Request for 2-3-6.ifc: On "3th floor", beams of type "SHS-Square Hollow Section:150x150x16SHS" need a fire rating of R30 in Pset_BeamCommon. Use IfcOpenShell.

First a look at what the model holds.

```python
import ifcopenshell
import ifcopenshell.util.element

model = ifcopenshell.open("2-3-6.ifc")
print(model.schema)
storey = next(s for s in model.by_type("IfcBuildingStorey") if s.Name == "3th floor")
beams = [e for e in ifcopenshell.util.element.get_decomposition(storey) if e.is_a("IfcBeam")]
seen = {}
for e in beams:
    element_type = ifcopenshell.util.element.get_type(e)
    key = (element_type.Name if element_type != e and element_type else None, ifcopenshell.util.element.get_pset(e, "Pset_BeamCommon", "FireRating"))
    seen[key] = seen.get(key, 0) + 1
for (name, value), count in sorted(seen.items(), key=str):
    print(count, "x", name, "|", value)
```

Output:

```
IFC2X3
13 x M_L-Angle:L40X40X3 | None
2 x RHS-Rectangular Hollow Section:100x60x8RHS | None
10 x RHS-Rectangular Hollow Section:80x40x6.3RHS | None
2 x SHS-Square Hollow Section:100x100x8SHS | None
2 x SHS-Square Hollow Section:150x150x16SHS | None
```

```python
import ifcopenshell
import ifcopenshell.api.pset
import ifcopenshell.util.element

model = ifcopenshell.open("2-3-6.ifc")

storey = next(s for s in model.by_type("IfcBuildingStorey") if s.Name == "3th floor")
beams = [e for e in ifcopenshell.util.element.get_decomposition(storey) if e.is_a("IfcBeam")]

count = 0
for e in beams:
    element_type = ifcopenshell.util.element.get_type(e)
    if element_type in (None, e) or element_type.Name != "SHS-Square Hollow Section:150x150x16SHS":
        continue
    # add_pset returns the element's existing set when there is one.
    pset = ifcopenshell.api.pset.add_pset(model, product=e, name="Pset_BeamCommon")
    ifcopenshell.api.pset.edit_pset(model, pset=pset, properties={"FireRating": "R30"})
    count += 1

print(count, "beams updated")

model.write("2-3-6_v2.ifc")
```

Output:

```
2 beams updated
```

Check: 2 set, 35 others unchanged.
